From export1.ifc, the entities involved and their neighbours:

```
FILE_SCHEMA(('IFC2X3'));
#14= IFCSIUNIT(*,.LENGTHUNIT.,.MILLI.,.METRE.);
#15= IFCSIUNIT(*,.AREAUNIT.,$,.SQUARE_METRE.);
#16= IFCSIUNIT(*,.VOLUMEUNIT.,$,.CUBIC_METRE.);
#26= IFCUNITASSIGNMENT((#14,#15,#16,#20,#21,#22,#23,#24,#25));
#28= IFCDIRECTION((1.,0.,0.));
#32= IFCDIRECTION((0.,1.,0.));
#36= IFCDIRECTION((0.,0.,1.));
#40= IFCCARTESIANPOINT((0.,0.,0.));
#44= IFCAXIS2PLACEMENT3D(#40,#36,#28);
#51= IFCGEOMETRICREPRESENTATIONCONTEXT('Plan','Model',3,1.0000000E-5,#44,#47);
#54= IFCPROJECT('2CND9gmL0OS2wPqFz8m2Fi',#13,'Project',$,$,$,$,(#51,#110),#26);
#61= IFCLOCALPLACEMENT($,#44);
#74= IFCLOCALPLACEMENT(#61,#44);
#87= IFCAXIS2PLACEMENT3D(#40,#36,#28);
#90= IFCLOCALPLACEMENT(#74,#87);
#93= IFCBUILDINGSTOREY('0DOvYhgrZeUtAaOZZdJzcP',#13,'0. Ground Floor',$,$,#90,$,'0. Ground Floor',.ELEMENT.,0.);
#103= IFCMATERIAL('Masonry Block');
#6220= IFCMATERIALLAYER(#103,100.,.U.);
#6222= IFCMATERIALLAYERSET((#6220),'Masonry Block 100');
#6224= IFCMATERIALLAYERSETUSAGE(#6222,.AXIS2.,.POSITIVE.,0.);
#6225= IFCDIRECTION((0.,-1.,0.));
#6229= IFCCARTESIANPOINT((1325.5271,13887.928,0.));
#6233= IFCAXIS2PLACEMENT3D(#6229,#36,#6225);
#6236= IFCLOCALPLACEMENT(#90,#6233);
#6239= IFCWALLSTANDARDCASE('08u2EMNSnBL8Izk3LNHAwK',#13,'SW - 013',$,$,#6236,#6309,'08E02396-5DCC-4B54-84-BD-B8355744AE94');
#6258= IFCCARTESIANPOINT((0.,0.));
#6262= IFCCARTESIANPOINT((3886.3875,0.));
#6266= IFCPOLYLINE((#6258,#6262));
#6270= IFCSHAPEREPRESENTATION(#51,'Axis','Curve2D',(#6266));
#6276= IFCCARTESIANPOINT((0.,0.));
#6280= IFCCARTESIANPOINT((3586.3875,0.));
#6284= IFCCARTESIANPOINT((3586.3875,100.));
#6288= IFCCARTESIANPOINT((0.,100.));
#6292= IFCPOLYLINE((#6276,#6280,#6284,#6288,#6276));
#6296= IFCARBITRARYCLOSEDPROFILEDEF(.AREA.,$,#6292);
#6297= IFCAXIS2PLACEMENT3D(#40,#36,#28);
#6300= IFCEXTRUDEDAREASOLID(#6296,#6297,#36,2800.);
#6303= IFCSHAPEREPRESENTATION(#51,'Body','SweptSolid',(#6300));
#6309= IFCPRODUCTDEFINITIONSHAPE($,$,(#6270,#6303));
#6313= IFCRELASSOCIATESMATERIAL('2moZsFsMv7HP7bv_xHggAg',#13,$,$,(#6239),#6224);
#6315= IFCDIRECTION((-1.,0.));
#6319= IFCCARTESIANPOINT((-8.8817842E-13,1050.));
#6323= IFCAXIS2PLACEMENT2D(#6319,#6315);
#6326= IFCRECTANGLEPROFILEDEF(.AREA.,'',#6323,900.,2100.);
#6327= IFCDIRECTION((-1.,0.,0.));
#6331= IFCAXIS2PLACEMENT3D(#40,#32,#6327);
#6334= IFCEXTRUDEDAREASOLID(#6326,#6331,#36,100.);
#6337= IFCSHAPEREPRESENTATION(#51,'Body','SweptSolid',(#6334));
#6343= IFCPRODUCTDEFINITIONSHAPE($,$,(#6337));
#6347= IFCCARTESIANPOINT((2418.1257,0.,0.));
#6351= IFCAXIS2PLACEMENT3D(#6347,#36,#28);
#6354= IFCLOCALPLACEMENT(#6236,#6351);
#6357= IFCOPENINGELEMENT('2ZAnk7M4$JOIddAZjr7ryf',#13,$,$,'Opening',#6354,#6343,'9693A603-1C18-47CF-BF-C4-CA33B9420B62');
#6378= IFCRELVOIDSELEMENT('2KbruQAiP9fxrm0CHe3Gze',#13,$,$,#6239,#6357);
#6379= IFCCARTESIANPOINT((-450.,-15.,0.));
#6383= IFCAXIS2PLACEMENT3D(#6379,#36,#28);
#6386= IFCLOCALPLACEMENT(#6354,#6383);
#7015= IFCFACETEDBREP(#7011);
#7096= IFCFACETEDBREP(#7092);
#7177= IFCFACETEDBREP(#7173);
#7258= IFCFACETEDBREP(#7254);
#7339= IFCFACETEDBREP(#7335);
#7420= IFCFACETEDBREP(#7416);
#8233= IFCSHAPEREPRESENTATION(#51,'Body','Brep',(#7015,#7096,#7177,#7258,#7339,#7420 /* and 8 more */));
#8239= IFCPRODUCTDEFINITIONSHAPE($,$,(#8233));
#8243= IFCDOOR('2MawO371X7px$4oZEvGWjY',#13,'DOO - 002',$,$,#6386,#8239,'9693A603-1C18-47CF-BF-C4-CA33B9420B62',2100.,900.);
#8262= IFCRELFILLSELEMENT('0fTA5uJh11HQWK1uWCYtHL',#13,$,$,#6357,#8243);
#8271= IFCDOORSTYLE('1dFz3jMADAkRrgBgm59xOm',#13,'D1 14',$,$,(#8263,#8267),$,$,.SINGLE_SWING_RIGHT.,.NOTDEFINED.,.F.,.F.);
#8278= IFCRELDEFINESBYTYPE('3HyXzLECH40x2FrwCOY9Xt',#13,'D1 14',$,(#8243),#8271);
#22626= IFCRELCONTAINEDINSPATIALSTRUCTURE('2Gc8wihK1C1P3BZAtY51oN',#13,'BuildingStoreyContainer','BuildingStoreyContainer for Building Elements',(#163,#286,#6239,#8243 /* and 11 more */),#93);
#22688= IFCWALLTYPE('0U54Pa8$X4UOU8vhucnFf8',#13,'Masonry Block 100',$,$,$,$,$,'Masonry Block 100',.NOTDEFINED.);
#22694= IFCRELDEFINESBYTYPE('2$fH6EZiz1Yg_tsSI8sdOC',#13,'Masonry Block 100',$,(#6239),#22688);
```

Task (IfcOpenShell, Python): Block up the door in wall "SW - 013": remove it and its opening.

```python
import ifcopenshell
import ifcopenshell.api.feature
import ifcopenshell.api.root
import ifcopenshell.geom
import ifcopenshell.util.shape

model = ifcopenshell.open("export1.ifc")
settings = ifcopenshell.geom.settings()


def volume(element):
    """Net volume in cubic metres, openings subtracted."""
    shape = ifcopenshell.geom.create_shape(settings, element)
    return ifcopenshell.util.shape.get_volume(shape.geometry)


door = model.by_guid("2MawO371X7px$4oZEvGWjY")
opening = door.FillsVoids[0].RelatingOpeningElement
wall = opening.VoidsElements[0].RelatingBuildingElement
before = volume(wall)

ifcopenshell.api.root.remove_product(model, product=door)
ifcopenshell.api.feature.remove_feature(model, feature=opening)

after = volume(wall)

print(f"wall volume {before:.3f} -> {after:.3f} m3")

model.write("export1-out.ifc")
```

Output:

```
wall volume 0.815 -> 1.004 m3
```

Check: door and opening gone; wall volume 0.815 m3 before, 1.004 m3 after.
